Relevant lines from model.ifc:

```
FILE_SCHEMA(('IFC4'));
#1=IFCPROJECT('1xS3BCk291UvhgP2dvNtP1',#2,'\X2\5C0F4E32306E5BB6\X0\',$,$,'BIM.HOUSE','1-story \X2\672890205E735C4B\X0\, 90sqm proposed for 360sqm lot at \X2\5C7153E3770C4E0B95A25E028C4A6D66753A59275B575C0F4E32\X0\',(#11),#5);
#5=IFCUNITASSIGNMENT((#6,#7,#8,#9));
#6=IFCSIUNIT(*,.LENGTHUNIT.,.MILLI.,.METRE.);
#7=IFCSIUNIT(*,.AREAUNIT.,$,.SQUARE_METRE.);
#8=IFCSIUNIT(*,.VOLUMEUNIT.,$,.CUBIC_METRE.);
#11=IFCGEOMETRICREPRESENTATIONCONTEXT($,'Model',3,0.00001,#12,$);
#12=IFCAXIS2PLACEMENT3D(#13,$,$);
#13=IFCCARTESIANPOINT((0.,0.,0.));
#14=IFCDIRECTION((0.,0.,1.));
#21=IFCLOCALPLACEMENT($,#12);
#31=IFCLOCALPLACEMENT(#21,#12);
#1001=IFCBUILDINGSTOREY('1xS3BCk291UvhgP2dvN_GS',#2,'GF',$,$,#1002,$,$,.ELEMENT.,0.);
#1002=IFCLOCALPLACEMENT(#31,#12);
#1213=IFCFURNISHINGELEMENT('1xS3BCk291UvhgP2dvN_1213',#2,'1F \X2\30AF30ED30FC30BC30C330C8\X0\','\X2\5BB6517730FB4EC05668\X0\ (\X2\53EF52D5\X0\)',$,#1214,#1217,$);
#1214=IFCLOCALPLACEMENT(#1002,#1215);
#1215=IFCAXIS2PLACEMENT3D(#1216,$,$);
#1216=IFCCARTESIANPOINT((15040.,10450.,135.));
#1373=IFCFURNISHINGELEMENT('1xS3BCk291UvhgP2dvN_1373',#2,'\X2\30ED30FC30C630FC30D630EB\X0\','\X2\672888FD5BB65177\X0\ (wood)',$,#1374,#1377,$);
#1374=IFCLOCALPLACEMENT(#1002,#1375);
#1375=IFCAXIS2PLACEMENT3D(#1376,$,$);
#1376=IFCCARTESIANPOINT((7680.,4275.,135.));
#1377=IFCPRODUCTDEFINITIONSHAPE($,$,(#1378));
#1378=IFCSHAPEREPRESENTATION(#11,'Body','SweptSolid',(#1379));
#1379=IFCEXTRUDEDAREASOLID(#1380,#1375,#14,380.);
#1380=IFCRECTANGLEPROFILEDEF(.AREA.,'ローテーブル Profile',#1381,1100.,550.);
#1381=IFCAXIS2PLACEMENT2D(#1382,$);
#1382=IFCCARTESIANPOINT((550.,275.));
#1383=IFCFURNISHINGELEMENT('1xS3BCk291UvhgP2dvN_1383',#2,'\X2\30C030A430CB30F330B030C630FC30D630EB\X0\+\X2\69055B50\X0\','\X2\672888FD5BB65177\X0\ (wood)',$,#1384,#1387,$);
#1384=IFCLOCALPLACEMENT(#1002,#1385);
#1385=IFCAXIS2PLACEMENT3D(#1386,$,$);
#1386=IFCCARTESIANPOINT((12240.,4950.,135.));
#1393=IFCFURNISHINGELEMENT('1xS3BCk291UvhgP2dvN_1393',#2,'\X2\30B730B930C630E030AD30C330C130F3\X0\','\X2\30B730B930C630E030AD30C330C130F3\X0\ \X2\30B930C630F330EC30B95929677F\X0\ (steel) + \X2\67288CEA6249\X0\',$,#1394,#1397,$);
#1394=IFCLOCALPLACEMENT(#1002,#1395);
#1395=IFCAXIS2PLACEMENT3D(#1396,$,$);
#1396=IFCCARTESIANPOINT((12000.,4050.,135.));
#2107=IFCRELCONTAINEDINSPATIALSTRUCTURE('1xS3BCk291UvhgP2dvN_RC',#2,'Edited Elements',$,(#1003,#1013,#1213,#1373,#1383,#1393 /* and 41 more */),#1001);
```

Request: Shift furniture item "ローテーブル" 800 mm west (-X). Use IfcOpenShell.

```python
import ifcopenshell
import ifcopenshell.api.geometry
import ifcopenshell.util.placement
import ifcopenshell.util.unit

model = ifcopenshell.open("model.ifc")
unit_scale = ifcopenshell.util.unit.calculate_unit_scale(model)

item = model.by_guid("1xS3BCk291UvhgP2dvN_1373")
matrix = ifcopenshell.util.placement.get_local_placement(item.ObjectPlacement)
matrix[0, 3] -= 0.8 / unit_scale
ifcopenshell.api.geometry.edit_object_placement(model, product=item, matrix=matrix, is_si=False)

print(ifcopenshell.util.placement.get_local_placement(item.ObjectPlacement).round(3) + 0.0)

model.write("model_rev.ifc")
```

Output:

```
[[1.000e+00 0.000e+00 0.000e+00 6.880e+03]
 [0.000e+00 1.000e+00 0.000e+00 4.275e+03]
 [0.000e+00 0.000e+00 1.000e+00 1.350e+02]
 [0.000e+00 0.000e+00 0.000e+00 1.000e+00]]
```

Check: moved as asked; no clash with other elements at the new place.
